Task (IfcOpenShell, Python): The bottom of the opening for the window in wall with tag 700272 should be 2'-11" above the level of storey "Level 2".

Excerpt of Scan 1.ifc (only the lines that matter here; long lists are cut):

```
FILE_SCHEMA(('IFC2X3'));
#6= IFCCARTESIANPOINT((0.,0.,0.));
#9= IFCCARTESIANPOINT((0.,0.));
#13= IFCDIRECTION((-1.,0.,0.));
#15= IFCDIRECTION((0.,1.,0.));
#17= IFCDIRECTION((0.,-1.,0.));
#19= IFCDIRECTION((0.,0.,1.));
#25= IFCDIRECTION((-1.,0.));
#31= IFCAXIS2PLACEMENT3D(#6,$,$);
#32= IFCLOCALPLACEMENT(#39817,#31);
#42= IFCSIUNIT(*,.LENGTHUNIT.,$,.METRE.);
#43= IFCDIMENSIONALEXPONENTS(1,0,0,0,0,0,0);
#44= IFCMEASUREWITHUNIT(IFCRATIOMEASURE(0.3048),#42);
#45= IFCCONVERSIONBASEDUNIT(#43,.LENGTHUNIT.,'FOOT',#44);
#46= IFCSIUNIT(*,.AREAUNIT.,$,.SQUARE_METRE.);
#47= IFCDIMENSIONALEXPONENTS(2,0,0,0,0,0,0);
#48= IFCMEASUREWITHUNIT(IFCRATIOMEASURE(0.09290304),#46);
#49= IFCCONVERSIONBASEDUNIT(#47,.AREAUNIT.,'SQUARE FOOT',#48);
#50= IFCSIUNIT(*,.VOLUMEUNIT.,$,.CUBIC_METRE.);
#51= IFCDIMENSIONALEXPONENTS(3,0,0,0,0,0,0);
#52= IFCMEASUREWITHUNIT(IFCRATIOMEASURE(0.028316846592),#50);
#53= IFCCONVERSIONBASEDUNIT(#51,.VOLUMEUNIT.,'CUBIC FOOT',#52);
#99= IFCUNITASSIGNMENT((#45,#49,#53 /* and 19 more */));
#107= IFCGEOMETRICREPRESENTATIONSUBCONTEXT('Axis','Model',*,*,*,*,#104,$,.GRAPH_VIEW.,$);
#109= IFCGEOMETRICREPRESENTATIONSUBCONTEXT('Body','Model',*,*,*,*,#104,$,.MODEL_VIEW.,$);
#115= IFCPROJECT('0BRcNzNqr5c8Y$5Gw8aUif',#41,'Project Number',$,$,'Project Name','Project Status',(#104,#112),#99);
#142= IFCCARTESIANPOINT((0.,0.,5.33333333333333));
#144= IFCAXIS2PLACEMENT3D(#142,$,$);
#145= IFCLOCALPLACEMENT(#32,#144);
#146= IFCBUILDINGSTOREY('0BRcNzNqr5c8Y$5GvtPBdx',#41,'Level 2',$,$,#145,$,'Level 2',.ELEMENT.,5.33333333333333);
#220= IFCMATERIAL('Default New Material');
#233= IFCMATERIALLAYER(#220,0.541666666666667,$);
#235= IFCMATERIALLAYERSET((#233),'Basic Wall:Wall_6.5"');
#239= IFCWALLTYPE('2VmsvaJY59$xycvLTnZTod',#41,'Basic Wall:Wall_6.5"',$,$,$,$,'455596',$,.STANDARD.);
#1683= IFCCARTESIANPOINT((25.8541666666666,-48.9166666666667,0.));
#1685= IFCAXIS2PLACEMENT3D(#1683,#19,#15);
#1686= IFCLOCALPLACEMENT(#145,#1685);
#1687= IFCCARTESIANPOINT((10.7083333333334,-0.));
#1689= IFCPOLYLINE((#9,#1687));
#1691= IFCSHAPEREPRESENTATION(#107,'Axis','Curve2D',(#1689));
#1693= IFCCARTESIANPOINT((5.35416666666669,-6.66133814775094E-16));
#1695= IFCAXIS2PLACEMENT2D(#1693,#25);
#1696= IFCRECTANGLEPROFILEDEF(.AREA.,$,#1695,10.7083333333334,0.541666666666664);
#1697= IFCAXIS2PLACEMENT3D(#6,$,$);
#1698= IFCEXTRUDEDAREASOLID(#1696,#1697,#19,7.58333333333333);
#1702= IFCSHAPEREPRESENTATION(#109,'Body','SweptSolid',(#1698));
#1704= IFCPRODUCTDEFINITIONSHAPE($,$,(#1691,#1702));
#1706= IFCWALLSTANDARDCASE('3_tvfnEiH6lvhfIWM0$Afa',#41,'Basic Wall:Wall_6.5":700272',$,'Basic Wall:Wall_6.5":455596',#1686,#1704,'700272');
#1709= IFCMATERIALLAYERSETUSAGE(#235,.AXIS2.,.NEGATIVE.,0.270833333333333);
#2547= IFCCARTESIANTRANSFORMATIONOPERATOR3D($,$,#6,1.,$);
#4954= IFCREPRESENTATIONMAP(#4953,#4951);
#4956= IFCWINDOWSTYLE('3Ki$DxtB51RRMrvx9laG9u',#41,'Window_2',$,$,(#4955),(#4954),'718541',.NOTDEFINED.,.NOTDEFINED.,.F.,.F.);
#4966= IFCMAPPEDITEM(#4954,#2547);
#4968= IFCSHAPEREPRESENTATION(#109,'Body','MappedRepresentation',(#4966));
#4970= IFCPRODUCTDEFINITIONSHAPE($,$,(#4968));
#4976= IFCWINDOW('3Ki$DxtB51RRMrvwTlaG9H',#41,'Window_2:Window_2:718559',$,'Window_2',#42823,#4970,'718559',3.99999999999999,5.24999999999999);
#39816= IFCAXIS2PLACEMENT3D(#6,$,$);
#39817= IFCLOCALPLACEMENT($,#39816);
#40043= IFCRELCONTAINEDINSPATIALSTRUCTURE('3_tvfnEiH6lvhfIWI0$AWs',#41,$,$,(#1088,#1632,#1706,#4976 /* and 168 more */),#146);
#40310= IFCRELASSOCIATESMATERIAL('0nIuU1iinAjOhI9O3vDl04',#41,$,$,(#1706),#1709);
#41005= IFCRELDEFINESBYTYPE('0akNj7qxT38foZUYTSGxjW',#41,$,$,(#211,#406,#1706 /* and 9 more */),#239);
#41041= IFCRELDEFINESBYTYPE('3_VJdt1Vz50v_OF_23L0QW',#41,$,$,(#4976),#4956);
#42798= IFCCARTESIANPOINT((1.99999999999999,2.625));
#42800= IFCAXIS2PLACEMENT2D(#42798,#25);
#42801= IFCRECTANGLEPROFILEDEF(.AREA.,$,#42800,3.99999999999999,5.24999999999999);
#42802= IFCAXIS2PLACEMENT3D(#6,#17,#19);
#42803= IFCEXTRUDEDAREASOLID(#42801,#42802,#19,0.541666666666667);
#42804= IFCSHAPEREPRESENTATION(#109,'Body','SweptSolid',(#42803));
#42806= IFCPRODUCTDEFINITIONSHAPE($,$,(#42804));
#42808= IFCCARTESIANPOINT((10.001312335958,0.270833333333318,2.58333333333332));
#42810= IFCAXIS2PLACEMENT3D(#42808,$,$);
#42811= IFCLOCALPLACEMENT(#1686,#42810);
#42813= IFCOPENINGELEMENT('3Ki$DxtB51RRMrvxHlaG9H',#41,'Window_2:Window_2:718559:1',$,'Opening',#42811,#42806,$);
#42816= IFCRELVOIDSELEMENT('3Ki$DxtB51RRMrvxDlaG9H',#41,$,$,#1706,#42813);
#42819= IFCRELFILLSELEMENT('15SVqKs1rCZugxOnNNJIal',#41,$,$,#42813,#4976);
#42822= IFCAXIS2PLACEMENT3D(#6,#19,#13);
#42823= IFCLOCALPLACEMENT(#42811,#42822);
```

```python
import numpy as np
import ifcopenshell
import ifcopenshell.api.geometry
import ifcopenshell.geom
import ifcopenshell.util.element
import ifcopenshell.util.placement
import ifcopenshell.util.shape
import ifcopenshell.util.unit

model = ifcopenshell.open("Scan 1.ifc")
unit_scale = ifcopenshell.util.unit.calculate_unit_scale(model)

window = model.by_guid("3Ki$DxtB51RRMrvwTlaG9H")
opening = window.FillsVoids[0].RelatingOpeningElement
storey = ifcopenshell.util.element.get_container(window, ifc_class="IfcBuildingStorey")
level = ifcopenshell.util.placement.get_local_placement(storey.ObjectPlacement)[2, 3]

# The opening's origin need not be at the sill, so measure its lowest point.
shape = ifcopenshell.geom.create_shape(ifcopenshell.geom.settings(), opening)
bottom = ifcopenshell.util.shape.get_shape_bottom_elevation(shape, shape.geometry) / unit_scale
dz = level + 35 * 0.0254 / unit_scale - bottom

shift = np.array([0.0, 0.0, dz])
# The window is placed relative to its opening, so it follows when the opening moves.
matrix = ifcopenshell.util.placement.get_local_placement(opening.ObjectPlacement)
matrix[:3, 3] += shift
ifcopenshell.api.geometry.edit_object_placement(
    model, product=opening, matrix=matrix, is_si=False, should_transform_children=True
)

print(f"moved by {dz * unit_scale:+.3f} m")

model.write("Scan 1_v2.ifc")
```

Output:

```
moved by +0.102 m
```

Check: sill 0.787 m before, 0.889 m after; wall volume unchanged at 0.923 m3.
